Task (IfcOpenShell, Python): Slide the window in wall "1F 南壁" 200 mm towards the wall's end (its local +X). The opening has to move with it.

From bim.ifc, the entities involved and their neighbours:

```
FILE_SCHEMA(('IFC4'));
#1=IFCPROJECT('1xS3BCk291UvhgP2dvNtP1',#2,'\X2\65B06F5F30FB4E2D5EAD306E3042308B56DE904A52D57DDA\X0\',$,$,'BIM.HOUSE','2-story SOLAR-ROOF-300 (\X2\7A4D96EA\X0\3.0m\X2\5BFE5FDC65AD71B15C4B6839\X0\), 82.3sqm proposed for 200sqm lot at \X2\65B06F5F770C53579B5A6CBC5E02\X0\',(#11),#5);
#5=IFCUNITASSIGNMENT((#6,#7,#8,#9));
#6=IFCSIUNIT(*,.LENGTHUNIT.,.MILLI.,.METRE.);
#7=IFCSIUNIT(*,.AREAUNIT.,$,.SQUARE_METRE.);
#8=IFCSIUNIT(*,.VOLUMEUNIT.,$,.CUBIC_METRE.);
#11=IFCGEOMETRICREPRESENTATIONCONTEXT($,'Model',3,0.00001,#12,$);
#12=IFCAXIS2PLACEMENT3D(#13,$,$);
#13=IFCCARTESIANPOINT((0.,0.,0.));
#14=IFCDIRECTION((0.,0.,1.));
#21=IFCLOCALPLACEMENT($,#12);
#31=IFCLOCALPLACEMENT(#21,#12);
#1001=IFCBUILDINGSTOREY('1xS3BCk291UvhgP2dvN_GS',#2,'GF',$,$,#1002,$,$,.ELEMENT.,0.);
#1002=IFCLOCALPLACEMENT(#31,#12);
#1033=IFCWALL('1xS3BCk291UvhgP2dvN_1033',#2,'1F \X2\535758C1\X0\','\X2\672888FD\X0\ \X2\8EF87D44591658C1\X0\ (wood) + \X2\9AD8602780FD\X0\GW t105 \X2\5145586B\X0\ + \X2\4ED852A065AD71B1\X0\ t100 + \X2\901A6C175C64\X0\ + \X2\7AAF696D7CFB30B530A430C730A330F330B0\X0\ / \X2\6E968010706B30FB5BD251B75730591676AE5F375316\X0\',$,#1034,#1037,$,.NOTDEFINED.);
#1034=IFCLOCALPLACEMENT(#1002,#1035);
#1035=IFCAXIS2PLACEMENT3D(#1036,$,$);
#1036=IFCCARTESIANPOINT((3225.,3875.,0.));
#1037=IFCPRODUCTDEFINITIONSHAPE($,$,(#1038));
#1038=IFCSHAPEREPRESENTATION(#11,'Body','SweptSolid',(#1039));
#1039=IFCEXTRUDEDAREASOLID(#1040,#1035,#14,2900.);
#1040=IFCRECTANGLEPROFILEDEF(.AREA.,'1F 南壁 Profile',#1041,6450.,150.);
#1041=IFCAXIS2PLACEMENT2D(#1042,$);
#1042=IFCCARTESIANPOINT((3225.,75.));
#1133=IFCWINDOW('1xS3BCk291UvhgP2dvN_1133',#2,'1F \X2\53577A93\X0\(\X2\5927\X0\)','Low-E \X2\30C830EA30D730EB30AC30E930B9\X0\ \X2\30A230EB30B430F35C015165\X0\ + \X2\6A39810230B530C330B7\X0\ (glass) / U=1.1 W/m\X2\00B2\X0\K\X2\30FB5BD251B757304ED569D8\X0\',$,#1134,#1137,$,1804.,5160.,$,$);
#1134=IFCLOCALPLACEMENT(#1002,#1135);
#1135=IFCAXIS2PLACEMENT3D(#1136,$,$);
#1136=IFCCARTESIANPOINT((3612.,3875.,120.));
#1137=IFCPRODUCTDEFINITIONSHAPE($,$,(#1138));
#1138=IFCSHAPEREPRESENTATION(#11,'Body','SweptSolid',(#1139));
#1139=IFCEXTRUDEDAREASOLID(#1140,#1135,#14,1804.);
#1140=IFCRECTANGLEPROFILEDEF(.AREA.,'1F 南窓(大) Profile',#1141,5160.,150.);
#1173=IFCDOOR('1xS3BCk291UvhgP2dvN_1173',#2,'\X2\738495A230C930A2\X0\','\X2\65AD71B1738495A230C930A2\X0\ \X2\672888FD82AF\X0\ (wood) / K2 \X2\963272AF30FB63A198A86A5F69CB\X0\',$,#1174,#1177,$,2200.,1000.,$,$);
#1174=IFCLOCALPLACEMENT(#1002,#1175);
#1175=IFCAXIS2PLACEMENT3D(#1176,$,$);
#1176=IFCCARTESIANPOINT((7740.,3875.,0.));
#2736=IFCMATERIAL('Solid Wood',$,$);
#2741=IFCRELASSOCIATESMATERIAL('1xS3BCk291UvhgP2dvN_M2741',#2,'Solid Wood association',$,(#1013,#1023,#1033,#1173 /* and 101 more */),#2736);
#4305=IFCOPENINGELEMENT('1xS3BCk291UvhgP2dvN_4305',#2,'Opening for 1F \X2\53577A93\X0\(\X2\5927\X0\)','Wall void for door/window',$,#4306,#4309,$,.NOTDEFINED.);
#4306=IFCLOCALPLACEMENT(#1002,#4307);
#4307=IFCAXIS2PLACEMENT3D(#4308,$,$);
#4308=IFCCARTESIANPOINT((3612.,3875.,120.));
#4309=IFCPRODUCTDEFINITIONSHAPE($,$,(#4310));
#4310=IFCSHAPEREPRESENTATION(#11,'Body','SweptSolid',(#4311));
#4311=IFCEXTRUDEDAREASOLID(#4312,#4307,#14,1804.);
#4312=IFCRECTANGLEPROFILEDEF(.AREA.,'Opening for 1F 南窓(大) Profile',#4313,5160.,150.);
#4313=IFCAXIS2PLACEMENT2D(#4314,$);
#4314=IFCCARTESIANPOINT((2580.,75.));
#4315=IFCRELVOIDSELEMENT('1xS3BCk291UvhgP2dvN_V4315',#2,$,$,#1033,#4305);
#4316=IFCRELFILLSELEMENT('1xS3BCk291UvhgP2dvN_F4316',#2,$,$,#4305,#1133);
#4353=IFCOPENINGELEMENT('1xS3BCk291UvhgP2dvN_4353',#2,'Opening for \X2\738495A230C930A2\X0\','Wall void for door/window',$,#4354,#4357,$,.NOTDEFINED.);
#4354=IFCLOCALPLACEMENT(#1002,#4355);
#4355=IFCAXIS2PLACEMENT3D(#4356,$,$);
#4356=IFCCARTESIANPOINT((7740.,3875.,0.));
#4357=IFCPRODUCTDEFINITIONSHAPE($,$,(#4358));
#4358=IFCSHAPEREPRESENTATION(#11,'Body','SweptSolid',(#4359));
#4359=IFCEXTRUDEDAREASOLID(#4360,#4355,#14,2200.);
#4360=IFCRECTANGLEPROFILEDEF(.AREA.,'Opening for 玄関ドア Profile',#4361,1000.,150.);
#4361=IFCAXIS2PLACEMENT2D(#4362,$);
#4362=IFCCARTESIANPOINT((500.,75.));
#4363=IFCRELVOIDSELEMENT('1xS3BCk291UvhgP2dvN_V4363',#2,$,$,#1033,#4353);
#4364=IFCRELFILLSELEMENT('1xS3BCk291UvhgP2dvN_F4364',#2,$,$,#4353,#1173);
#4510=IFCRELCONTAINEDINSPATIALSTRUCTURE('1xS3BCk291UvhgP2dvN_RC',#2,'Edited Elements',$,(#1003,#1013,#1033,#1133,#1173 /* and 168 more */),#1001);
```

```python
import ifcopenshell
import ifcopenshell.api.geometry
import ifcopenshell.util.placement
import ifcopenshell.util.unit

model = ifcopenshell.open("bim.ifc")
unit_scale = ifcopenshell.util.unit.calculate_unit_scale(model)

window = model.by_guid("1xS3BCk291UvhgP2dvN_1133")
opening = window.FillsVoids[0].RelatingOpeningElement
wall = opening.VoidsElements[0].RelatingBuildingElement

wall_matrix = ifcopenshell.util.placement.get_local_placement(wall.ObjectPlacement)
shift = wall_matrix[:3, 0] * 0.2 / unit_scale
before = ifcopenshell.util.placement.get_local_placement(window.ObjectPlacement)[:3, 3].copy()

# The window is not placed relative to its opening, so move both.
for product in (opening, window):
    matrix = ifcopenshell.util.placement.get_local_placement(product.ObjectPlacement)
    matrix[:3, 3] += shift
    ifcopenshell.api.geometry.edit_object_placement(model, product=product, matrix=matrix, is_si=False)

after = ifcopenshell.util.placement.get_local_placement(window.ObjectPlacement)[:3, 3]
print("window moved by", (after - before).round(3) + 0.0)

model.write("bim_edited.ifc")
```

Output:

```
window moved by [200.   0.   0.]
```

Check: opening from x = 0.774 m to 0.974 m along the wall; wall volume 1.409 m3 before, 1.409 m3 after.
